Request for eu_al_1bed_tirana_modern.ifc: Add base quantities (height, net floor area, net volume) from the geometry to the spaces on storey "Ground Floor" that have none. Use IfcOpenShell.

First a look at what the model holds.

```python
import ifcopenshell
import ifcopenshell.util.element
import ifcopenshell.util.unit

model = ifcopenshell.open("eu_al_1bed_tirana_modern.ifc")
print(model.schema)
for unit_type in ("LENGTHUNIT", "AREAUNIT", "VOLUMEUNIT"):
    print(unit_type, ifcopenshell.util.unit.calculate_unit_scale(model, unit_type))
storey = next(s for s in model.by_type("IfcBuildingStorey") if s.Name == "Ground Floor")
spaces = [e for e in ifcopenshell.util.element.get_decomposition(storey) if e.is_a("IfcSpace")]
for e in sorted(spaces, key=lambda e: e.id()):
    print(e.id(), e.is_a(), e.Name, list(ifcopenshell.util.element.get_psets(e, qtos_only=True)), sep=" | ")
```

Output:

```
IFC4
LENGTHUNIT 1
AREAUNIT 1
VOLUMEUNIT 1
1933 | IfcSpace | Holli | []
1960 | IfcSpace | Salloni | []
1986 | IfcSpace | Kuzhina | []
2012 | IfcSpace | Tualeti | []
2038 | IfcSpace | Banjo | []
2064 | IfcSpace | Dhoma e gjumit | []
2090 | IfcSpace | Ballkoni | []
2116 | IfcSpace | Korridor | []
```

```python
import ifcopenshell
import ifcopenshell.api.pset
import ifcopenshell.geom
import ifcopenshell.util.element
import ifcopenshell.util.shape
import ifcopenshell.util.unit

model = ifcopenshell.open("eu_al_1bed_tirana_modern.ifc")
unit_scale = ifcopenshell.util.unit.calculate_unit_scale(model)
area_scale = ifcopenshell.util.unit.calculate_unit_scale(model, "AREAUNIT")
volume_scale = ifcopenshell.util.unit.calculate_unit_scale(model, "VOLUMEUNIT")
settings = ifcopenshell.geom.settings()

storey = next(s for s in model.by_type("IfcBuildingStorey") if s.Name == "Ground Floor")
spaces = [e for e in ifcopenshell.util.element.get_decomposition(storey) if e.is_a("IfcSpace")]

for e in sorted(spaces, key=lambda e: e.id()):
    if ifcopenshell.util.element.get_psets(e, qtos_only=True, should_inherit=False):
        continue
    # Geometry comes back in metres, in the element's own axes.
    shape = ifcopenshell.geom.create_shape(settings, e)
    values = {
        "Height": ifcopenshell.util.shape.get_z(shape.geometry) / unit_scale,
        "NetFloorArea": ifcopenshell.util.shape.get_footprint_area(shape.geometry) / area_scale,
        "NetVolume": ifcopenshell.util.shape.get_volume(shape.geometry) / volume_scale,
    }
    qto = ifcopenshell.api.pset.add_qto(model, product=e, name="Qto_SpaceBaseQuantities")
    ifcopenshell.api.pset.edit_qto(model, qto=qto, properties=values)
    print(e.id(), {k: round(v, 3) for k, v in values.items()})

model.write("eu_al_1bed_tirana_modern_edited.ifc")
```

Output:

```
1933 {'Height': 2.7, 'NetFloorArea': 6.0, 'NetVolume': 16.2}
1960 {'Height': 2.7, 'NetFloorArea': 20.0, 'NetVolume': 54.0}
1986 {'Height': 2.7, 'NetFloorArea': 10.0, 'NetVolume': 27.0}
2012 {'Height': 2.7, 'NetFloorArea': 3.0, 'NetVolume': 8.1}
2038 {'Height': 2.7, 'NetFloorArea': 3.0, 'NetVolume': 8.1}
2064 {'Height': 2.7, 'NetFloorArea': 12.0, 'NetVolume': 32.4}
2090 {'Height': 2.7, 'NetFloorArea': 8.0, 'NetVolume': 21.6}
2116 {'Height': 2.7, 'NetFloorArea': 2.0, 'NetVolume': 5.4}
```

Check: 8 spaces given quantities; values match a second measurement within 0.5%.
